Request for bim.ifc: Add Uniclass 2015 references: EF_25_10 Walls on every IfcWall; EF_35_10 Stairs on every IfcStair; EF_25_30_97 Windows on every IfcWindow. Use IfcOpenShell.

First a look at what the model holds.

```python
import ifcopenshell

model = ifcopenshell.open("bim.ifc")
print(model.schema)
print("classifications:", [c.Name for c in model.by_type("IfcClassification")])
for ifc_class in ("IfcDoor", "IfcRoof", "IfcStair", "IfcWall", "IfcWindow"):
    print(ifc_class, len(model.by_type(ifc_class)))
```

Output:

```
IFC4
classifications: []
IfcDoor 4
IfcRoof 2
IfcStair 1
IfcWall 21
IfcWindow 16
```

```python
import ifcopenshell
import ifcopenshell.api.classification

model = ifcopenshell.open("bim.ifc")

system = ifcopenshell.api.classification.add_classification(model, classification="Uniclass 2015")

codes = {
    "IfcWall": ("EF_25_10", "Walls"),
    "IfcStair": ("EF_35_10", "Stairs"),
    "IfcWindow": ("EF_25_30_97", "Windows"),
}
for ifc_class, (code, name) in codes.items():
    products = model.by_type(ifc_class)
    ifcopenshell.api.classification.add_reference(
        model, products=products, classification=system, identification=code, name=name
    )
    print(code, len(products))

model.write("bim_rev.ifc")
```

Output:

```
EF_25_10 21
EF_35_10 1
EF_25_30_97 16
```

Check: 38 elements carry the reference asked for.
